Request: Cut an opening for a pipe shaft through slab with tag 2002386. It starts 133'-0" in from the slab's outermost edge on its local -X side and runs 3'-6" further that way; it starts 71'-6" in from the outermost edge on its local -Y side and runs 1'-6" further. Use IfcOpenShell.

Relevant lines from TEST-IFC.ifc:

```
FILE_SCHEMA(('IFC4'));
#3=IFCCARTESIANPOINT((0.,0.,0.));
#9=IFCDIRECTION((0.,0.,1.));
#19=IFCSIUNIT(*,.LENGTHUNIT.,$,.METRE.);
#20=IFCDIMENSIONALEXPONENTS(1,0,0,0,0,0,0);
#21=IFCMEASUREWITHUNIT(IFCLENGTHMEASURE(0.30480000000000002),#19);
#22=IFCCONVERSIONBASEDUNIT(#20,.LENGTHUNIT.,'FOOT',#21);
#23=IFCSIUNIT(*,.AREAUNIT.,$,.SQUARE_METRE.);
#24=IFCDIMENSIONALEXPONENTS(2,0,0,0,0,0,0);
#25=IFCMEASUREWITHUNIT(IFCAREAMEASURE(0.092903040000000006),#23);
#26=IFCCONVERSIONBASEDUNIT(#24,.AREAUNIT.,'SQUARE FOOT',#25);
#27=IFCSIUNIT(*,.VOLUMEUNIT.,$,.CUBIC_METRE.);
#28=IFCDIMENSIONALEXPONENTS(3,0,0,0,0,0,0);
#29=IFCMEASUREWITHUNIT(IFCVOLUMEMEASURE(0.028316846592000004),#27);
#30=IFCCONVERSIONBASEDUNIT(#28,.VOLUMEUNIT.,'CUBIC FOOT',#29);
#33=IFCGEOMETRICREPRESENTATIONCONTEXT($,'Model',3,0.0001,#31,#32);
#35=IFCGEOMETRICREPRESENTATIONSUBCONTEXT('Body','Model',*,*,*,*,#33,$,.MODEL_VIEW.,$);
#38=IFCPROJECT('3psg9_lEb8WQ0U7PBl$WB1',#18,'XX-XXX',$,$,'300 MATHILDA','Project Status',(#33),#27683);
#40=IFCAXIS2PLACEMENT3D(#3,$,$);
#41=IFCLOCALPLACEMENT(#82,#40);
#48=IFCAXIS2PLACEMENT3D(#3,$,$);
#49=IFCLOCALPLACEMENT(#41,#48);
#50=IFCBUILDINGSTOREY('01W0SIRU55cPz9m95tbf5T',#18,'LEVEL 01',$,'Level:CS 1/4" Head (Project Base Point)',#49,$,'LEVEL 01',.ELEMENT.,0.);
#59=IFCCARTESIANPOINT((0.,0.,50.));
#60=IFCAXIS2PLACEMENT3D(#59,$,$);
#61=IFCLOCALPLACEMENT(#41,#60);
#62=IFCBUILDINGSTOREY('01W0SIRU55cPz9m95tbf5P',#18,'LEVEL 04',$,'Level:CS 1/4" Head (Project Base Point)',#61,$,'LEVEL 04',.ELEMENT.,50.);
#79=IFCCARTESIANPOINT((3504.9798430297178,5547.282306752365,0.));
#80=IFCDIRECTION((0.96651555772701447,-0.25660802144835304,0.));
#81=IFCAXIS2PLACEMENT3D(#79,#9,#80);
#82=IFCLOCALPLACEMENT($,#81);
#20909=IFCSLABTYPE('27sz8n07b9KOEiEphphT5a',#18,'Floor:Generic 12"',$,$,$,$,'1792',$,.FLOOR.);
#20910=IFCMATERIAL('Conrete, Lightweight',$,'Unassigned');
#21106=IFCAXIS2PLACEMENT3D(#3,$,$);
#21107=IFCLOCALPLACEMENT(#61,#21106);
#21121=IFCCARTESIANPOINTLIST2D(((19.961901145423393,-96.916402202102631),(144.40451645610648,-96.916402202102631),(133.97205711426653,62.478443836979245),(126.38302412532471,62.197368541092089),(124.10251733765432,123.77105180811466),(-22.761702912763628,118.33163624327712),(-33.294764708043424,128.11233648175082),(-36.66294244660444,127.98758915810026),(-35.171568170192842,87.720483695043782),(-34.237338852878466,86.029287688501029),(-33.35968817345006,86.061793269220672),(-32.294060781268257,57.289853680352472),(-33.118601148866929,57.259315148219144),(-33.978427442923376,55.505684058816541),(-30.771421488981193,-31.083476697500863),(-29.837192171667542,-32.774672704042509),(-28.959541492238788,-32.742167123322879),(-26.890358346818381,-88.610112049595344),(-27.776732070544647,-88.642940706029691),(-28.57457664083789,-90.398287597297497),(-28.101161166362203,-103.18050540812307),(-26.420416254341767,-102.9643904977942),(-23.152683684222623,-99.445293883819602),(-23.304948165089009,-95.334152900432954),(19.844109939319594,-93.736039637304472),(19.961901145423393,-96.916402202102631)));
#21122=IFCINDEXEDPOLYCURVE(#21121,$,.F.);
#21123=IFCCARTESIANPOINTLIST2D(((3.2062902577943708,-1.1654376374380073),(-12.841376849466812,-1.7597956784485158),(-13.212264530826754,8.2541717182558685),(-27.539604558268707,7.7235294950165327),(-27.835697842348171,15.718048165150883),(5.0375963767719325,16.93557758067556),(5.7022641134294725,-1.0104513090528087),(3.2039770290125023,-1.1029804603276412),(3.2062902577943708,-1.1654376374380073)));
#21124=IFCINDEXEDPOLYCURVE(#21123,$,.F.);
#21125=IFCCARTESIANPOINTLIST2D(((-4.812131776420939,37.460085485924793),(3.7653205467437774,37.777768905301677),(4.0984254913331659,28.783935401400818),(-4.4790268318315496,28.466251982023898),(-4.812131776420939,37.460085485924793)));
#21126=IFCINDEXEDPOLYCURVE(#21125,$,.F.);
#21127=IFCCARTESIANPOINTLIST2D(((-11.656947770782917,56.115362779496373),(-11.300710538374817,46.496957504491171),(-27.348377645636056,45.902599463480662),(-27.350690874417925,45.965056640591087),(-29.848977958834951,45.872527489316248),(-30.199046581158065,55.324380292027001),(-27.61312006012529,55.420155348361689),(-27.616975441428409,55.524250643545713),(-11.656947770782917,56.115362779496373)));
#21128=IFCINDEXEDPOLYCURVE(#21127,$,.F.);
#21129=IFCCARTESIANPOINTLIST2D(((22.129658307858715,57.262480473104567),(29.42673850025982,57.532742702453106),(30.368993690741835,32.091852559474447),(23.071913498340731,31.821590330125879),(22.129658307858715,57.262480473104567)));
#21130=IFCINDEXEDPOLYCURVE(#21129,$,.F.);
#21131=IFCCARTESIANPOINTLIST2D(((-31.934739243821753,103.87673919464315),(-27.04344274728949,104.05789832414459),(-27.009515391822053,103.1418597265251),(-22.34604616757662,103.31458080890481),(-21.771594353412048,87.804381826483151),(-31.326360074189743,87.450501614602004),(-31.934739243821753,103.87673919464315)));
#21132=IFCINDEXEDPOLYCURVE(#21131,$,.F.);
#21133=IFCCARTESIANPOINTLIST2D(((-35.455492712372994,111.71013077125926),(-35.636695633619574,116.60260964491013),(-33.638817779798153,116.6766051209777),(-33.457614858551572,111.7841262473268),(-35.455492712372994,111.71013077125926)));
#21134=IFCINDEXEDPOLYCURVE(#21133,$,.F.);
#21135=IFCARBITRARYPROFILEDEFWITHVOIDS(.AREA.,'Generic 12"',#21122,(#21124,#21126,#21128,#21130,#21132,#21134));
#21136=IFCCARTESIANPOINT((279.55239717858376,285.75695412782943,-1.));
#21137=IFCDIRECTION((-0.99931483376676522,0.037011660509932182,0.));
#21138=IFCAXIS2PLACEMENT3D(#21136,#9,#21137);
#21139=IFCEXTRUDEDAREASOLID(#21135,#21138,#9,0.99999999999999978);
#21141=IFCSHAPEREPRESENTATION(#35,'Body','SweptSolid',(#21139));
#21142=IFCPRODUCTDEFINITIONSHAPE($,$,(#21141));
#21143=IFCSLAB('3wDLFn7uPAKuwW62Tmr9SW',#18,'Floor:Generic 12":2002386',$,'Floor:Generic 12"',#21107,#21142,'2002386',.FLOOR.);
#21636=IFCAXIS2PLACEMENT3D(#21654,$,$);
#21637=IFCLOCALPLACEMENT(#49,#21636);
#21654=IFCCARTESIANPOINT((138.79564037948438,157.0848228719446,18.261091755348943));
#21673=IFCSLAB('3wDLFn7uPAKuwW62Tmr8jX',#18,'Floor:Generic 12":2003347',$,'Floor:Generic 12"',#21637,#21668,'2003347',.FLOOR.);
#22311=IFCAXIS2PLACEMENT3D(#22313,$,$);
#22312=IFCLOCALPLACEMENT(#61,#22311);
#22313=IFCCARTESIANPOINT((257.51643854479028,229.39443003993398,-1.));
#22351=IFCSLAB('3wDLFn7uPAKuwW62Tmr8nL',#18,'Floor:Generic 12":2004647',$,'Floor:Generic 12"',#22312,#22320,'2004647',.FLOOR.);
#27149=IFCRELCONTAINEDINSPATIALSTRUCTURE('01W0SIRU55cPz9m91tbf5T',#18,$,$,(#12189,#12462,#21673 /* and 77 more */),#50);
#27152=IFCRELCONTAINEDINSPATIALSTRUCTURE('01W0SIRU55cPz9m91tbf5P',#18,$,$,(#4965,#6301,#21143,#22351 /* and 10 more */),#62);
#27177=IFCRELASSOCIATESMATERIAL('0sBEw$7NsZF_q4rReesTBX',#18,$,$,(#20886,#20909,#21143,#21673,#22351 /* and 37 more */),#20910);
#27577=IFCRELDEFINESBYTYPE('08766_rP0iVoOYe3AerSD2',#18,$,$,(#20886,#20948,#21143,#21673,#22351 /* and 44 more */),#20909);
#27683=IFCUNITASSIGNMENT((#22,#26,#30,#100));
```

```python
import numpy as np
import ifcopenshell
import ifcopenshell.api.feature
import ifcopenshell.api.geometry
import ifcopenshell.api.root
import ifcopenshell.geom
import ifcopenshell.util.placement
import ifcopenshell.util.representation
import ifcopenshell.util.shape
import ifcopenshell.util.unit

model = ifcopenshell.open("TEST-IFC.ifc")
unit_scale = ifcopenshell.util.unit.calculate_unit_scale(model)
settings = ifcopenshell.geom.settings()


def volume(element):
    """Net volume in cubic metres, openings subtracted."""
    shape = ifcopenshell.geom.create_shape(settings, element)
    return ifcopenshell.util.shape.get_volume(shape.geometry)


slab = model.by_guid("3wDLFn7uPAKuwW62Tmr9SW")
before = volume(slab)

# Extent in the slab's own axes, in metres. The edges named are its -X and -Y sides.
slab_shape = ifcopenshell.geom.create_shape(settings, slab)
vertices = ifcopenshell.util.shape.get_vertices(slab_shape.geometry)
x_min, y_min, bottom = vertices.min(axis=0)
top = vertices[:, 2].max()

opening = ifcopenshell.api.root.create_entity(model, ifc_class="IfcOpeningElement", name="Pipe shaft opening", predefined_type="OPENING")
context = ifcopenshell.util.representation.get_context(model, "Model", "Body", "MODEL_VIEW")
width, depth = 1.0668, 0.4572
outline = [(0.0, 0.0), (width, 0.0), (width, depth), (0.0, depth), (0.0, 0.0)]
# Overshoot both faces by 50 mm so the cut is clean.
shape = ifcopenshell.api.geometry.add_slab_representation(
    model, context=context, depth=top - bottom + 0.1, polyline=outline
)
ifcopenshell.api.geometry.assign_representation(model, product=opening, representation=shape)

matrix = ifcopenshell.util.placement.get_local_placement(slab.ObjectPlacement)
matrix[:, 3] = matrix @ np.append(np.array([x_min + 40.5384, y_min + 21.7932, bottom - 0.05]) / unit_scale, 1.0)
ifcopenshell.api.geometry.edit_object_placement(model, product=opening, matrix=matrix, is_si=False)
ifcopenshell.api.feature.add_feature(model, feature=opening, element=slab)

after = volume(slab)

print(f"slab volume {before:.3f} -> {after:.3f} m3")

model.write("TEST-IFC_updated.ifc")
```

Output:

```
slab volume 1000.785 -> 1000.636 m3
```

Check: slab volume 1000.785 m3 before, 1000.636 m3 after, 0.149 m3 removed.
